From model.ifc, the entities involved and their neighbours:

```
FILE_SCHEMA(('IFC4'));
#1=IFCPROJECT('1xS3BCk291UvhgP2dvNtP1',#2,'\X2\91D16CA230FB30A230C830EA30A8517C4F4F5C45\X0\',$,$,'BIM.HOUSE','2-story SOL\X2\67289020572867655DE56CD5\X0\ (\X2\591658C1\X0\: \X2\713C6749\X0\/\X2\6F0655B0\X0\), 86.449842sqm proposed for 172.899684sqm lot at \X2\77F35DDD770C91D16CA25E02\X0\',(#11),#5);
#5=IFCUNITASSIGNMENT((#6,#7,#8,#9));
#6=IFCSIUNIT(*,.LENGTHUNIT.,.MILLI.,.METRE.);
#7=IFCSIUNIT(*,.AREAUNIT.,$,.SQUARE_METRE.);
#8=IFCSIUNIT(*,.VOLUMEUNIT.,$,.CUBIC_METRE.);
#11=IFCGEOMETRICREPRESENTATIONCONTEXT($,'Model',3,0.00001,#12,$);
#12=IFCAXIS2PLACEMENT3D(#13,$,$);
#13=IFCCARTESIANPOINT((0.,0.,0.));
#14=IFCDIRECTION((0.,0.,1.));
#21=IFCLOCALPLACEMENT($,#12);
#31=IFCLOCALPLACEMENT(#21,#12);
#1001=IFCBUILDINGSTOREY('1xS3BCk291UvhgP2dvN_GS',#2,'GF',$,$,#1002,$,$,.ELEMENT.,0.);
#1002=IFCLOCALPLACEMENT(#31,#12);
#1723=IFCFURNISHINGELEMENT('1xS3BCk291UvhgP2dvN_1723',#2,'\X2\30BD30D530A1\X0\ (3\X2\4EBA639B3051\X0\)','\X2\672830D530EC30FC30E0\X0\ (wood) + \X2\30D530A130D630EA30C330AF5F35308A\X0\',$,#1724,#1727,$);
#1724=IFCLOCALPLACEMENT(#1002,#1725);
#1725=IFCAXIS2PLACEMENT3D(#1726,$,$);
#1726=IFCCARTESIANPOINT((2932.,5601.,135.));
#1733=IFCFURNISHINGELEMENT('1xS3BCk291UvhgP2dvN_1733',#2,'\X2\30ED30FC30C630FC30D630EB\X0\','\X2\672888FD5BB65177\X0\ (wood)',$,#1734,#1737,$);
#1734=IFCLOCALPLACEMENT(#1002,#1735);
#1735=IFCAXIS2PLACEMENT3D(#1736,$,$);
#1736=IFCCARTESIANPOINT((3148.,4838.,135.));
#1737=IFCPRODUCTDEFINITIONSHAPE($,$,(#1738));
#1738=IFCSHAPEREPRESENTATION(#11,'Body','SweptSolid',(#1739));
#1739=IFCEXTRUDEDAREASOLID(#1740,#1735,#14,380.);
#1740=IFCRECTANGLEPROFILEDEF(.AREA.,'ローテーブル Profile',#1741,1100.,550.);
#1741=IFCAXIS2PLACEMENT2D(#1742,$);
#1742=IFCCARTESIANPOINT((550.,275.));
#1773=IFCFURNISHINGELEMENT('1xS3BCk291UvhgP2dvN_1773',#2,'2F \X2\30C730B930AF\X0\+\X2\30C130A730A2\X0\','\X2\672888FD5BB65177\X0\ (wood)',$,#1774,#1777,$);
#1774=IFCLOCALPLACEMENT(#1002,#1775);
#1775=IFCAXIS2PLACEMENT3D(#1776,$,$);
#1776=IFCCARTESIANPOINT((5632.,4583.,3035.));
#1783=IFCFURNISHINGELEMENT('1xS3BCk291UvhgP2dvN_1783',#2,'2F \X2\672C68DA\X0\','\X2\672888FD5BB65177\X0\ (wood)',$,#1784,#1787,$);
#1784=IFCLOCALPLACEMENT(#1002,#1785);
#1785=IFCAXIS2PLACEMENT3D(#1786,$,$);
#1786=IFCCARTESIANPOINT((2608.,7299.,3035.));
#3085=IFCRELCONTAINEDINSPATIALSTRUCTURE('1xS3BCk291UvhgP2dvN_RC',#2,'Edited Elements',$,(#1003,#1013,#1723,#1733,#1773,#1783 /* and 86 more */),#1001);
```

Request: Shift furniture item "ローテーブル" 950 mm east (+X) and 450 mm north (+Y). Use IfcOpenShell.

```python
import ifcopenshell
import ifcopenshell.api.geometry
import ifcopenshell.util.placement
import ifcopenshell.util.unit

model = ifcopenshell.open("model.ifc")
unit_scale = ifcopenshell.util.unit.calculate_unit_scale(model)

item = model.by_guid("1xS3BCk291UvhgP2dvN_1733")
matrix = ifcopenshell.util.placement.get_local_placement(item.ObjectPlacement)
matrix[0, 3] += 0.95 / unit_scale
matrix[1, 3] += 0.45 / unit_scale
ifcopenshell.api.geometry.edit_object_placement(model, product=item, matrix=matrix, is_si=False)

print(ifcopenshell.util.placement.get_local_placement(item.ObjectPlacement).round(3) + 0.0)

model.write("model-out.ifc")
```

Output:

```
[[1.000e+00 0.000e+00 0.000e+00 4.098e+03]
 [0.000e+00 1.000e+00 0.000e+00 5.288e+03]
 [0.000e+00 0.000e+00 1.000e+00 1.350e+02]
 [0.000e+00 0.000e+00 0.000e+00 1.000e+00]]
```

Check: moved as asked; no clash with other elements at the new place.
